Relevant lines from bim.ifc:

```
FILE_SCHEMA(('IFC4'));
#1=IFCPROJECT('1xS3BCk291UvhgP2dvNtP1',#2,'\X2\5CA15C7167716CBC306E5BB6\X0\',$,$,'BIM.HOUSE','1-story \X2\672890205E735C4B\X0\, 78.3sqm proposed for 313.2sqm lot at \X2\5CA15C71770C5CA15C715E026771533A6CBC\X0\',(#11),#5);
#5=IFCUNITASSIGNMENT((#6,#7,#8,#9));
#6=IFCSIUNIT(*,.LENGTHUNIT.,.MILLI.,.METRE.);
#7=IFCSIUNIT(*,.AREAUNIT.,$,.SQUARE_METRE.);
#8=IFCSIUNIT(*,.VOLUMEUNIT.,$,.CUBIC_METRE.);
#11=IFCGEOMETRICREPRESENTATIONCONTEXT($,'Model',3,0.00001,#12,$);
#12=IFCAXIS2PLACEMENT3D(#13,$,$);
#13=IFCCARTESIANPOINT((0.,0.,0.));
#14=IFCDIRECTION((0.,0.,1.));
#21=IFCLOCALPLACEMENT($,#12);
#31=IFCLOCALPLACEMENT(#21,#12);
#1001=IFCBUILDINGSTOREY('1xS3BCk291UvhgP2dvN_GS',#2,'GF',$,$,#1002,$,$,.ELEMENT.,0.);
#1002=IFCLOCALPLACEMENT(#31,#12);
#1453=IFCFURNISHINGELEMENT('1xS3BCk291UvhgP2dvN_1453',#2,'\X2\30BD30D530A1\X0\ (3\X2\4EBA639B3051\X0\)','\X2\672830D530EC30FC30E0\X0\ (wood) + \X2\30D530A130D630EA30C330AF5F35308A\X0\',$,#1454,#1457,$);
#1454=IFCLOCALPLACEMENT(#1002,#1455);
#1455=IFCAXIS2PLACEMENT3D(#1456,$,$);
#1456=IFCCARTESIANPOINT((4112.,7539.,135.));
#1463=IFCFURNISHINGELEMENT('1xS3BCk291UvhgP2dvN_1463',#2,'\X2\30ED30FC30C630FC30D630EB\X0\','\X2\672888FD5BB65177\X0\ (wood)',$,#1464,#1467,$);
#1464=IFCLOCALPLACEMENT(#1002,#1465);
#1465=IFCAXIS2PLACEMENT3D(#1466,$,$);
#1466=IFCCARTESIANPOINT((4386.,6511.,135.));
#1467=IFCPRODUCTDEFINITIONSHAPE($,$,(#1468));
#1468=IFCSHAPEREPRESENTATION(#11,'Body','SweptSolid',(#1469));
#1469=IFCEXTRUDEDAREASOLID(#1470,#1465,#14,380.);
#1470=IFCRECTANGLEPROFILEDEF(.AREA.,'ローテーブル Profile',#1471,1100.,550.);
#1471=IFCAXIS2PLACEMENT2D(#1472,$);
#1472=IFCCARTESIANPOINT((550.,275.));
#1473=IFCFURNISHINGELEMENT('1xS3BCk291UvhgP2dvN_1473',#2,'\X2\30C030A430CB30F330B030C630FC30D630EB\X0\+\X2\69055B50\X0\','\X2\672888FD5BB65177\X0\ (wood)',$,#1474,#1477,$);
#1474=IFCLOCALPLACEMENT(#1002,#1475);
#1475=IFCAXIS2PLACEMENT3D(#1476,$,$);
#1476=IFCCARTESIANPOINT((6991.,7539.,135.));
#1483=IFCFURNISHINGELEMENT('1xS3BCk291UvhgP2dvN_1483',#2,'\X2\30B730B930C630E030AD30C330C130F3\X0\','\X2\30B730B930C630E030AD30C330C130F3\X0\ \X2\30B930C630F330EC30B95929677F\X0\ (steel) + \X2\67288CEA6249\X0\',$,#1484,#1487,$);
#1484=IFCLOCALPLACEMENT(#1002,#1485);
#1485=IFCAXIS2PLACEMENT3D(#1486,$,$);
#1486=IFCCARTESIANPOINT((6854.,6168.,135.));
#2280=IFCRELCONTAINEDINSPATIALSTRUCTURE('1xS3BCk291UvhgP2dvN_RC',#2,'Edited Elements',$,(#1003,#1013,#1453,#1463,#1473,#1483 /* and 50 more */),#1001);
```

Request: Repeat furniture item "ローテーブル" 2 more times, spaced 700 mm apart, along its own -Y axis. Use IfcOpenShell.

```python
import ifcopenshell
import ifcopenshell.api.geometry
import ifcopenshell.api.root
import ifcopenshell.util.element
import ifcopenshell.util.placement
import ifcopenshell.util.unit

model = ifcopenshell.open("bim.ifc")
unit_scale = ifcopenshell.util.unit.calculate_unit_scale(model)


def reuse_history(source, copy):
    """copy_class also copies each property set's owner history, people and application; keep the originals."""
    for rel in copy.IsDefinedBy:
        if rel.is_a("IfcRelDefinesByProperties") and (history := rel.RelatingPropertyDefinition.OwnerHistory):
            rel.RelatingPropertyDefinition.OwnerHistory = source.OwnerHistory
            ifcopenshell.util.element.remove_deep2(model, history)


source = model.by_guid("1xS3BCk291UvhgP2dvN_1463")
base = ifcopenshell.util.placement.get_local_placement(source.ObjectPlacement)
step = -base[:3, 1] * 0.7 / unit_scale

for i in range(1, 3):
    copy = ifcopenshell.api.root.copy_class(model, product=source)
    copy.Representation = ifcopenshell.util.element.copy_deep(
        model, source.Representation, exclude=["IfcGeometricRepresentationContext", "IfcRepresentationMap"]
    )
    reuse_history(source, copy)
    matrix = base.copy()
    matrix[:3, 3] += i * step
    print("added at", matrix[:3, 3].round(3) + 0.0)
    ifcopenshell.api.geometry.edit_object_placement(model, product=copy, matrix=matrix, is_si=False)

model.write("bim_v2.ifc")
```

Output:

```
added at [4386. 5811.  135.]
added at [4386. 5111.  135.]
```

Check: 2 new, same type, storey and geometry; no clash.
